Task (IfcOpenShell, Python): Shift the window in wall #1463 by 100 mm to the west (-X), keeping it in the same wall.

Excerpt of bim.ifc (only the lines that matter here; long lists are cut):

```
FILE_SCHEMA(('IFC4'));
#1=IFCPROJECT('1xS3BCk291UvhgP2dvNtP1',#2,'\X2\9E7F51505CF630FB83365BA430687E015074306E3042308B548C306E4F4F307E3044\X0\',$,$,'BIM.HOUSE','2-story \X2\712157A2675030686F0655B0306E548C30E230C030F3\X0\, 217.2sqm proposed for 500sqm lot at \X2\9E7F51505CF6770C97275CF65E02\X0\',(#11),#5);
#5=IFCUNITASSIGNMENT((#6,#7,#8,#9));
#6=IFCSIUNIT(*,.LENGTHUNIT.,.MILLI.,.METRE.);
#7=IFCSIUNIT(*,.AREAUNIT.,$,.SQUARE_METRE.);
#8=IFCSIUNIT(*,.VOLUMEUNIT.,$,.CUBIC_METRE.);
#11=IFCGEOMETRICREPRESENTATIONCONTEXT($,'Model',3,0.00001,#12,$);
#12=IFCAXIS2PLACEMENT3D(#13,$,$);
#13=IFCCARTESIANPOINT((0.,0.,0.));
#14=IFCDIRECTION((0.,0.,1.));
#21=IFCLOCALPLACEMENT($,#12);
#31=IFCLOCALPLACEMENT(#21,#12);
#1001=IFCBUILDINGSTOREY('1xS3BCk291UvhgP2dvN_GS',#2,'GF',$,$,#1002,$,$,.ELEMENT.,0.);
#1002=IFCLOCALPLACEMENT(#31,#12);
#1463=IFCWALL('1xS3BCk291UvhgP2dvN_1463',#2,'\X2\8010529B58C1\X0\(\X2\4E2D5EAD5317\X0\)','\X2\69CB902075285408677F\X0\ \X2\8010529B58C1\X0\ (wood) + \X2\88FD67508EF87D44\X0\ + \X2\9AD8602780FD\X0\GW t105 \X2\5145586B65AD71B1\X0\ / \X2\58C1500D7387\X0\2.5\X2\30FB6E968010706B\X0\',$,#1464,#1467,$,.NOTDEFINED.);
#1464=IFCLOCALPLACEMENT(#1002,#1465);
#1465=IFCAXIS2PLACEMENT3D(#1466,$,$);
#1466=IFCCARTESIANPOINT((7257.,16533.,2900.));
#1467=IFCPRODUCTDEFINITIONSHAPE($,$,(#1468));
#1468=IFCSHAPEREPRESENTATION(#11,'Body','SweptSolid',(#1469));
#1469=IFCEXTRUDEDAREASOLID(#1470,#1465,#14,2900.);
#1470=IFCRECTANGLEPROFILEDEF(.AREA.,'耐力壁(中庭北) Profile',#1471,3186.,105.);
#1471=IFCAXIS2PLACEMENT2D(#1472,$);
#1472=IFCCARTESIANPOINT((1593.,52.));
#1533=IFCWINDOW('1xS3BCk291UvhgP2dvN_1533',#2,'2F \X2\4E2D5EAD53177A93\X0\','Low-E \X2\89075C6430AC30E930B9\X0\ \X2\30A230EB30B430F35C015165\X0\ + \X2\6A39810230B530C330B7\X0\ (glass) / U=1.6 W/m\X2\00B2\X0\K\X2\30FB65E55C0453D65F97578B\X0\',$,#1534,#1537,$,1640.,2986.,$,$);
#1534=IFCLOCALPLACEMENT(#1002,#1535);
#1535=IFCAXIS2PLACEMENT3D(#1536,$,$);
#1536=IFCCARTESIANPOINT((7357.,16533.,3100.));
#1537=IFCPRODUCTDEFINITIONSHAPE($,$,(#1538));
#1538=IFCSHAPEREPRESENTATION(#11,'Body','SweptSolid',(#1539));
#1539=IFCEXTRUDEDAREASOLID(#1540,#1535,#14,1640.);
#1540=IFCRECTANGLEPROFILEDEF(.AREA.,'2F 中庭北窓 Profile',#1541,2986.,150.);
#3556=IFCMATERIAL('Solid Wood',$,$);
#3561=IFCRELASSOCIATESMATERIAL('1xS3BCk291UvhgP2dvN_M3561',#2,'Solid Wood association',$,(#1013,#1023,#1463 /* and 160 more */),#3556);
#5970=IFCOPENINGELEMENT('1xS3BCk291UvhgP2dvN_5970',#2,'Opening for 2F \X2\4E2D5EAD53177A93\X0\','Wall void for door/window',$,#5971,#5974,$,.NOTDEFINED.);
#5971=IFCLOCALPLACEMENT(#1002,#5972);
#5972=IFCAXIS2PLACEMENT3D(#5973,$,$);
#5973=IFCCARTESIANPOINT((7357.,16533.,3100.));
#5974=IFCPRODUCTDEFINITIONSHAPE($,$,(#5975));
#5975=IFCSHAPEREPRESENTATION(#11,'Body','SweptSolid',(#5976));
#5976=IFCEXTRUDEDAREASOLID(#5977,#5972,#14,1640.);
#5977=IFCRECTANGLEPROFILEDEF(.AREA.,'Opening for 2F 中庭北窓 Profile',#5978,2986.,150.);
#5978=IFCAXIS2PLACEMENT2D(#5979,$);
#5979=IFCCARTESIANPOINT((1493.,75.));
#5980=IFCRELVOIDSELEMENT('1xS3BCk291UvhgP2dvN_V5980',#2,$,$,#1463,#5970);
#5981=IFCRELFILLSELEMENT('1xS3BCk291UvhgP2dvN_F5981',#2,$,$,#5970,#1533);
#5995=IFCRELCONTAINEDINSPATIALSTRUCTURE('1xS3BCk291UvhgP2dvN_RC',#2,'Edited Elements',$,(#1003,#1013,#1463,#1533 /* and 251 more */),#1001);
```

```python
import ifcopenshell
import ifcopenshell.api.geometry
import ifcopenshell.util.placement
import ifcopenshell.util.unit

model = ifcopenshell.open("bim.ifc")
unit_scale = ifcopenshell.util.unit.calculate_unit_scale(model)

window = model.by_guid("1xS3BCk291UvhgP2dvN_1533")
opening = window.FillsVoids[0].RelatingOpeningElement
wall = opening.VoidsElements[0].RelatingBuildingElement

wall_matrix = ifcopenshell.util.placement.get_local_placement(wall.ObjectPlacement)
shift = wall_matrix[:3, 0] * -0.1 / unit_scale
before = ifcopenshell.util.placement.get_local_placement(window.ObjectPlacement)[:3, 3].copy()

# The window is not placed relative to its opening, so move both.
for product in (opening, window):
    matrix = ifcopenshell.util.placement.get_local_placement(product.ObjectPlacement)
    matrix[:3, 3] += shift
    ifcopenshell.api.geometry.edit_object_placement(model, product=product, matrix=matrix, is_si=False)

after = ifcopenshell.util.placement.get_local_placement(window.ObjectPlacement)[:3, 3]
print("window moved by", (after - before).round(3) + 0.0)

model.write("bim-out.ifc")
```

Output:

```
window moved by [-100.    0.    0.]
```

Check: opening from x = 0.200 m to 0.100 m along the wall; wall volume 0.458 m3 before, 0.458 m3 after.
